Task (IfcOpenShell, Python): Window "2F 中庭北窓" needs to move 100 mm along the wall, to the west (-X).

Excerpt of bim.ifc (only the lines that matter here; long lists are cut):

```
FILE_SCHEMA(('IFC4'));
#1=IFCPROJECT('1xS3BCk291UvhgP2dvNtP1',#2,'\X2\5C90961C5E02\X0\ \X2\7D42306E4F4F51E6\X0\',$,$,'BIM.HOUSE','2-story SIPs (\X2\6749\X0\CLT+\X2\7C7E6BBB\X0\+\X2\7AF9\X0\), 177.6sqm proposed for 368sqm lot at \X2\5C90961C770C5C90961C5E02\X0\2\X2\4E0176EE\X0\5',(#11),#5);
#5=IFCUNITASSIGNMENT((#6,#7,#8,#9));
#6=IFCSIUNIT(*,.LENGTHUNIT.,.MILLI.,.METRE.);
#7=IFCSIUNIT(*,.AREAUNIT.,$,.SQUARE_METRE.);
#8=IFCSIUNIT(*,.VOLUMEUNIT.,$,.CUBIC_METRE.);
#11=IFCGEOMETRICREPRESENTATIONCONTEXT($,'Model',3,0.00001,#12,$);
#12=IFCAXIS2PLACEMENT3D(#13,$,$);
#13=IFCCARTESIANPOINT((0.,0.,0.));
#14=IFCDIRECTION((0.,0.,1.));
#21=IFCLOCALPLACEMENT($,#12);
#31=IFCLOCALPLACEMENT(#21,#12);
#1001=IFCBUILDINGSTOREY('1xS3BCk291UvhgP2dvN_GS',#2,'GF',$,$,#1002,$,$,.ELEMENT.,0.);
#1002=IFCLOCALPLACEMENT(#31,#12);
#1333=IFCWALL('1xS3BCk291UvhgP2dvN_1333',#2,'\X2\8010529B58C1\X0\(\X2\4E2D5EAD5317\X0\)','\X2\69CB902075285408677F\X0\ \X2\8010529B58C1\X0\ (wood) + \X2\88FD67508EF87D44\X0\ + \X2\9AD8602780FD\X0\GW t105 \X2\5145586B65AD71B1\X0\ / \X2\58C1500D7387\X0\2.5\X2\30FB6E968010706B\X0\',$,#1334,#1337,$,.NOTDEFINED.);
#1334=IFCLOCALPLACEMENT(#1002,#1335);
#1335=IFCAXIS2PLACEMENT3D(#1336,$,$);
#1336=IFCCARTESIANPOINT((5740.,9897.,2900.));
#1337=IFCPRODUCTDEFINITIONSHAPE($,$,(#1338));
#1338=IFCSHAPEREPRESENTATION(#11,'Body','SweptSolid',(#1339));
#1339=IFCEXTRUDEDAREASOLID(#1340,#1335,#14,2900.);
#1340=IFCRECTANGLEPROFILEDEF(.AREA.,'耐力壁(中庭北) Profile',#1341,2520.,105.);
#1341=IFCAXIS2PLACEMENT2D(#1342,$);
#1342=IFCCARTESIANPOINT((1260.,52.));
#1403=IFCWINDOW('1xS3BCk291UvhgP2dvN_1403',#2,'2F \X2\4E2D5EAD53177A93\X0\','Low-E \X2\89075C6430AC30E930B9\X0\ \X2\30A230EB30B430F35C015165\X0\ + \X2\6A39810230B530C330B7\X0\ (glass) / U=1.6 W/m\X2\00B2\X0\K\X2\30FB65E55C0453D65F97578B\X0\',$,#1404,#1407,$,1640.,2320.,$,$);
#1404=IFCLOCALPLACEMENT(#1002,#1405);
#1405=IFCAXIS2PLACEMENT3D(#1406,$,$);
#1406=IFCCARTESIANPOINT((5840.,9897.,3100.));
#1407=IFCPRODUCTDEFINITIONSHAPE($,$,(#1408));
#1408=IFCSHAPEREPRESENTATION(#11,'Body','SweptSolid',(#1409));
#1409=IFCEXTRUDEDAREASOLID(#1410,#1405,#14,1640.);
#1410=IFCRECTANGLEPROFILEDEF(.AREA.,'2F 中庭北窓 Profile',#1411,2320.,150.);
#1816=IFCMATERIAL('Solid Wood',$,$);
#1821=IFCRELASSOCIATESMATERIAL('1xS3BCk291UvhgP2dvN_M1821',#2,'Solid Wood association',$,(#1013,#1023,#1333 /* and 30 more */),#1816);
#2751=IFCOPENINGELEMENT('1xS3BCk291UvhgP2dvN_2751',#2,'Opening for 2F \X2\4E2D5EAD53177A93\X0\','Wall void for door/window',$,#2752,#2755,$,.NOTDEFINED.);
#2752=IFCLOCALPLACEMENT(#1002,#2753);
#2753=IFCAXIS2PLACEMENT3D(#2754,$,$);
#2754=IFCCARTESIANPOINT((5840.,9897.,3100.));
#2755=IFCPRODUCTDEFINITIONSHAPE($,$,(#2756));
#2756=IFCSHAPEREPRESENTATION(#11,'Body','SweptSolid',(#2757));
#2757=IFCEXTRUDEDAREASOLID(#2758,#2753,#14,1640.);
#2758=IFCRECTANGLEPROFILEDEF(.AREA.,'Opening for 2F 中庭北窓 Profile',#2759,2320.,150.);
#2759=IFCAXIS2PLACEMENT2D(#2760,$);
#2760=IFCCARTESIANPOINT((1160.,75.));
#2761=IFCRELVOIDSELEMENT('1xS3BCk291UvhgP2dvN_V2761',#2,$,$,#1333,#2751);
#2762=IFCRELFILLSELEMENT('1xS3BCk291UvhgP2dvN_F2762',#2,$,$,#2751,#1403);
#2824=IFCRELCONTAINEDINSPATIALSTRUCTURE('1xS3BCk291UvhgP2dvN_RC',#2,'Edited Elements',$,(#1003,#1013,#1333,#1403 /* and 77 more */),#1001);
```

```python
import ifcopenshell
import ifcopenshell.api.geometry
import ifcopenshell.util.placement

model = ifcopenshell.open("bim.ifc")

window = model.by_guid("1xS3BCk291UvhgP2dvN_1403")
opening = window.FillsVoids[0].RelatingOpeningElement
wall = opening.VoidsElements[0].RelatingBuildingElement

wall_matrix = ifcopenshell.util.placement.get_local_placement(wall.ObjectPlacement)
shift = wall_matrix[:3, 0] * -100.0
before = ifcopenshell.util.placement.get_local_placement(window.ObjectPlacement)[:3, 3].copy()

# The window is not placed relative to its opening, so move both.
for product in (opening, window):
    matrix = ifcopenshell.util.placement.get_local_placement(product.ObjectPlacement)
    matrix[:3, 3] += shift
    ifcopenshell.api.geometry.edit_object_placement(model, product=product, matrix=matrix, is_si=False)

after = ifcopenshell.util.placement.get_local_placement(window.ObjectPlacement)[:3, 3]
print("window moved by", (after - before).round(3) + 0.0)

model.write("bim-out.ifc")
```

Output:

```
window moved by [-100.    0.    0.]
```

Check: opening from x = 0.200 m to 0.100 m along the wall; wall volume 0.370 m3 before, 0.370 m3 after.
